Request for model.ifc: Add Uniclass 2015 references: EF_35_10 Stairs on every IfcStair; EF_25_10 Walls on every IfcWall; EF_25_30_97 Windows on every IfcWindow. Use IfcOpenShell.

First a look at what the model holds.

```python
import ifcopenshell

model = ifcopenshell.open("model.ifc")
print(model.schema)
print("classifications:", [c.Name for c in model.by_type("IfcClassification")])
for ifc_class in ("IfcDoor", "IfcRoof", "IfcStair", "IfcWall", "IfcWindow"):
    print(ifc_class, len(model.by_type(ifc_class)))
```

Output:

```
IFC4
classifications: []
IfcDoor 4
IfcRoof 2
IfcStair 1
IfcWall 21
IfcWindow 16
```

```python
import ifcopenshell
import ifcopenshell.api.classification

model = ifcopenshell.open("model.ifc")

system = ifcopenshell.api.classification.add_classification(model, classification="Uniclass 2015")

codes = {
    "IfcStair": ("EF_35_10", "Stairs"),
    "IfcWall": ("EF_25_10", "Walls"),
    "IfcWindow": ("EF_25_30_97", "Windows"),
}
for ifc_class, (code, name) in codes.items():
    products = model.by_type(ifc_class)
    ifcopenshell.api.classification.add_reference(
        model, products=products, classification=system, identification=code, name=name
    )
    print(code, len(products))

model.write("model_updated.ifc")
```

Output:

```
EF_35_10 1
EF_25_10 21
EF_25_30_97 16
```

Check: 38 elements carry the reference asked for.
